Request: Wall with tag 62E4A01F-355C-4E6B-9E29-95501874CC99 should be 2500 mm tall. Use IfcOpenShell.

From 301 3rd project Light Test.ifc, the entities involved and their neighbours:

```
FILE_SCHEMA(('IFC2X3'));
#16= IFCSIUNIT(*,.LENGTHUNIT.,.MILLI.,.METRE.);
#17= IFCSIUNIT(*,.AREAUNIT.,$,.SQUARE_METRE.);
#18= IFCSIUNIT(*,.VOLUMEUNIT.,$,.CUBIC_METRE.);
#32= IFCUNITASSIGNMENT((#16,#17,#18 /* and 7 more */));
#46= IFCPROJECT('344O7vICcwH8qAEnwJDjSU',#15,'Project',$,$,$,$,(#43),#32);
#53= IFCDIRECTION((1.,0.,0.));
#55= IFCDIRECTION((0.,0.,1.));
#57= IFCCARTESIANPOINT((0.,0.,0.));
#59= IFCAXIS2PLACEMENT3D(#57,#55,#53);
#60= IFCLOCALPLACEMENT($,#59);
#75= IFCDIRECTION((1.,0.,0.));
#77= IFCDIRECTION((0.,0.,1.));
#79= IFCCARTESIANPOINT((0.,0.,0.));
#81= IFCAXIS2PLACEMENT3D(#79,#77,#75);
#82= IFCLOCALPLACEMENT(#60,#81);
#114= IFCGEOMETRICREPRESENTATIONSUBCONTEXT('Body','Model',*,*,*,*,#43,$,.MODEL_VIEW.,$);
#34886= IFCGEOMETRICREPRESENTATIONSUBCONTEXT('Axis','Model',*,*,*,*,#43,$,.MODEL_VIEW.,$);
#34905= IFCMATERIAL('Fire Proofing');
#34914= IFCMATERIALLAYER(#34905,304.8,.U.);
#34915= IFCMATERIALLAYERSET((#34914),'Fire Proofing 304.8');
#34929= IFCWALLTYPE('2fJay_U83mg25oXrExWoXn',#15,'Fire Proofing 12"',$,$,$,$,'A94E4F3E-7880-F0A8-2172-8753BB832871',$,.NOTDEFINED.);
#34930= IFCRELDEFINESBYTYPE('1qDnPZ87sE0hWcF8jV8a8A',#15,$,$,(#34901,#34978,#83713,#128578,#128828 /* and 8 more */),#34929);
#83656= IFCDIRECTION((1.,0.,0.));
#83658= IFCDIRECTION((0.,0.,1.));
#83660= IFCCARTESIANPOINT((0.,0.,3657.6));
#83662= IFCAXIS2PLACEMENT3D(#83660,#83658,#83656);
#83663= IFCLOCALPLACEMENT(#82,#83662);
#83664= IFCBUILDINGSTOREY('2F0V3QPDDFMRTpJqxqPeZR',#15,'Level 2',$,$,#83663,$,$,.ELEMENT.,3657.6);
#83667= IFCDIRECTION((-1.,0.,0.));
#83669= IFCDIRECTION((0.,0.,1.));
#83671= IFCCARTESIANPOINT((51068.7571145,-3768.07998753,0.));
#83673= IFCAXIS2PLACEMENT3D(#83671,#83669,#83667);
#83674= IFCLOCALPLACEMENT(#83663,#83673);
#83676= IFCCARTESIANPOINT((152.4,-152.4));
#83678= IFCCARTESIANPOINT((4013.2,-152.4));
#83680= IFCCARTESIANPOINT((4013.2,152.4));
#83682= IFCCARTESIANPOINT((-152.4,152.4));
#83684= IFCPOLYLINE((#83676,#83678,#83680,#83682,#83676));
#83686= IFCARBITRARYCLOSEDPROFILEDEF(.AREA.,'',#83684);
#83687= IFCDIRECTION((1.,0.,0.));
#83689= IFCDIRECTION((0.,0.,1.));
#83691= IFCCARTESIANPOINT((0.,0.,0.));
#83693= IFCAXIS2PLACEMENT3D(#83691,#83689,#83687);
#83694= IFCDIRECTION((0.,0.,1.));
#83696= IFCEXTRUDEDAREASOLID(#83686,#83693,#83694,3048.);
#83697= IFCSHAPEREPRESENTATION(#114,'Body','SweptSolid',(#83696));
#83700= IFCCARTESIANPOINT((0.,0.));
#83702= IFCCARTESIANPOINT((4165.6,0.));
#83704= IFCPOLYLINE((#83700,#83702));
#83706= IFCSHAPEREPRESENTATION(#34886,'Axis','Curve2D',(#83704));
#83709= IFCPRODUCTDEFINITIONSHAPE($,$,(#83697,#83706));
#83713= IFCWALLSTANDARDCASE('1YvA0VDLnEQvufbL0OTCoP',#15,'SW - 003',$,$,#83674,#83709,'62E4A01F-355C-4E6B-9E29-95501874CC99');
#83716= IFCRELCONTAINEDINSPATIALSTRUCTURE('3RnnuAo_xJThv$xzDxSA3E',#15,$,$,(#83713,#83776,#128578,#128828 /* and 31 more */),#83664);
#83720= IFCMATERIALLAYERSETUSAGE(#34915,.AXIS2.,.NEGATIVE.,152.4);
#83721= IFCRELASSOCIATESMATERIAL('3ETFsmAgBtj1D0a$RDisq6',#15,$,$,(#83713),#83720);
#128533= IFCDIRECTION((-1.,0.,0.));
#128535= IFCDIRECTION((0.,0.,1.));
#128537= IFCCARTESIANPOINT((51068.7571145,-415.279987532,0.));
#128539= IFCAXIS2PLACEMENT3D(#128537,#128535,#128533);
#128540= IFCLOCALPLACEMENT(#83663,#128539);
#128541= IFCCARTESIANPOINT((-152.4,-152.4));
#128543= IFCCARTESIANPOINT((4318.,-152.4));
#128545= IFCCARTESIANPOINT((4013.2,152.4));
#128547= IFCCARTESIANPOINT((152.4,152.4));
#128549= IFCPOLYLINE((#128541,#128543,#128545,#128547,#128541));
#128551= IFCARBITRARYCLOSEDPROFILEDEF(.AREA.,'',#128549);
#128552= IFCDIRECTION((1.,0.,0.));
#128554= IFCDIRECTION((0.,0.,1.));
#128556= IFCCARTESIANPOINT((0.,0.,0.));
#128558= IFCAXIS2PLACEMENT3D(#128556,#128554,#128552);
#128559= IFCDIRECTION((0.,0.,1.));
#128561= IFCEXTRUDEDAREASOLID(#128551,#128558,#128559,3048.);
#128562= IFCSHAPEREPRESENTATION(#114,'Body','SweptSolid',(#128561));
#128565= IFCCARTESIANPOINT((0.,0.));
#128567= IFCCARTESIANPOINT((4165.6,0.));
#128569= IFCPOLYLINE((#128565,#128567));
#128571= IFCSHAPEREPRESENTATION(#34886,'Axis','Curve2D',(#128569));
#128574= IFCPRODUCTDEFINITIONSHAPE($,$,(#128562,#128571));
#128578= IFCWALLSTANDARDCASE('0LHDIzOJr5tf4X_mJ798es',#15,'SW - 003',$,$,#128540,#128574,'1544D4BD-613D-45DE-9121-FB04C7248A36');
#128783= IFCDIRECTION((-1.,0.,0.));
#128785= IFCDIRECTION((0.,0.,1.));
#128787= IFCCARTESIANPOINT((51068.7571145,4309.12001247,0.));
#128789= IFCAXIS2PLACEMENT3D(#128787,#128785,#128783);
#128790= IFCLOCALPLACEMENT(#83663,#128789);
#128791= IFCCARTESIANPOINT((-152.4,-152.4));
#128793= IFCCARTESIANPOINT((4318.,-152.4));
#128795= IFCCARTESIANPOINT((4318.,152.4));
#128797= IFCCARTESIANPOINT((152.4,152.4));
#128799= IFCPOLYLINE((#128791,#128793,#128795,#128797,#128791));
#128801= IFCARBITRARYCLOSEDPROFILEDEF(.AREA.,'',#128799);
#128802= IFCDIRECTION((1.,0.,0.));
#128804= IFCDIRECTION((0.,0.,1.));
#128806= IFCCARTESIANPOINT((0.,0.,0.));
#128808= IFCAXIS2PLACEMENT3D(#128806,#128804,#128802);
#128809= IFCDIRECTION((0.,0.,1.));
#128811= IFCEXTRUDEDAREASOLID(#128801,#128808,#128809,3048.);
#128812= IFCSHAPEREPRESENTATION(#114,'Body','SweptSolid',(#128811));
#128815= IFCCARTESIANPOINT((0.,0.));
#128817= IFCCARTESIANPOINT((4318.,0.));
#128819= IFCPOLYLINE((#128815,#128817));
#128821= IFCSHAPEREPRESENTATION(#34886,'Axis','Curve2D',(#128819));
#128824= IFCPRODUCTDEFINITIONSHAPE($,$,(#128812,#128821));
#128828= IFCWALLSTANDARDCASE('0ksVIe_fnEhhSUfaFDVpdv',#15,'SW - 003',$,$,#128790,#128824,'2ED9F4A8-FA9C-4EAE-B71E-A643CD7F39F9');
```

```python
import ifcopenshell
import ifcopenshell.geom
import ifcopenshell.util.representation
import ifcopenshell.util.shape
import ifcopenshell.util.unit

model = ifcopenshell.open("301 3rd project Light Test.ifc")
unit_scale = ifcopenshell.util.unit.calculate_unit_scale(model)
settings = ifcopenshell.geom.settings()


def volume(element):
    """Net volume in cubic metres, openings subtracted."""
    shape = ifcopenshell.geom.create_shape(settings, element)
    return ifcopenshell.util.shape.get_volume(shape.geometry)


wall = model.by_guid("1YvA0VDLnEQvufbL0OTCoP")
before = volume(wall)

body = ifcopenshell.util.representation.get_representation(wall, "Model", "Body")
solid = body.Items[0]
old_height = solid.Depth
solid.Depth = 2.5 / unit_scale
after = volume(wall)

print(f"height {old_height:g} -> {solid.Depth:g}, volume {before:.3f} -> {after:.3f} m3")

model.write("301 3rd project Light Test_edited.ifc")
```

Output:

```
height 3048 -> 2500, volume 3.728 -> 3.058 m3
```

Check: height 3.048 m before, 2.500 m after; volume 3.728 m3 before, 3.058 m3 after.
